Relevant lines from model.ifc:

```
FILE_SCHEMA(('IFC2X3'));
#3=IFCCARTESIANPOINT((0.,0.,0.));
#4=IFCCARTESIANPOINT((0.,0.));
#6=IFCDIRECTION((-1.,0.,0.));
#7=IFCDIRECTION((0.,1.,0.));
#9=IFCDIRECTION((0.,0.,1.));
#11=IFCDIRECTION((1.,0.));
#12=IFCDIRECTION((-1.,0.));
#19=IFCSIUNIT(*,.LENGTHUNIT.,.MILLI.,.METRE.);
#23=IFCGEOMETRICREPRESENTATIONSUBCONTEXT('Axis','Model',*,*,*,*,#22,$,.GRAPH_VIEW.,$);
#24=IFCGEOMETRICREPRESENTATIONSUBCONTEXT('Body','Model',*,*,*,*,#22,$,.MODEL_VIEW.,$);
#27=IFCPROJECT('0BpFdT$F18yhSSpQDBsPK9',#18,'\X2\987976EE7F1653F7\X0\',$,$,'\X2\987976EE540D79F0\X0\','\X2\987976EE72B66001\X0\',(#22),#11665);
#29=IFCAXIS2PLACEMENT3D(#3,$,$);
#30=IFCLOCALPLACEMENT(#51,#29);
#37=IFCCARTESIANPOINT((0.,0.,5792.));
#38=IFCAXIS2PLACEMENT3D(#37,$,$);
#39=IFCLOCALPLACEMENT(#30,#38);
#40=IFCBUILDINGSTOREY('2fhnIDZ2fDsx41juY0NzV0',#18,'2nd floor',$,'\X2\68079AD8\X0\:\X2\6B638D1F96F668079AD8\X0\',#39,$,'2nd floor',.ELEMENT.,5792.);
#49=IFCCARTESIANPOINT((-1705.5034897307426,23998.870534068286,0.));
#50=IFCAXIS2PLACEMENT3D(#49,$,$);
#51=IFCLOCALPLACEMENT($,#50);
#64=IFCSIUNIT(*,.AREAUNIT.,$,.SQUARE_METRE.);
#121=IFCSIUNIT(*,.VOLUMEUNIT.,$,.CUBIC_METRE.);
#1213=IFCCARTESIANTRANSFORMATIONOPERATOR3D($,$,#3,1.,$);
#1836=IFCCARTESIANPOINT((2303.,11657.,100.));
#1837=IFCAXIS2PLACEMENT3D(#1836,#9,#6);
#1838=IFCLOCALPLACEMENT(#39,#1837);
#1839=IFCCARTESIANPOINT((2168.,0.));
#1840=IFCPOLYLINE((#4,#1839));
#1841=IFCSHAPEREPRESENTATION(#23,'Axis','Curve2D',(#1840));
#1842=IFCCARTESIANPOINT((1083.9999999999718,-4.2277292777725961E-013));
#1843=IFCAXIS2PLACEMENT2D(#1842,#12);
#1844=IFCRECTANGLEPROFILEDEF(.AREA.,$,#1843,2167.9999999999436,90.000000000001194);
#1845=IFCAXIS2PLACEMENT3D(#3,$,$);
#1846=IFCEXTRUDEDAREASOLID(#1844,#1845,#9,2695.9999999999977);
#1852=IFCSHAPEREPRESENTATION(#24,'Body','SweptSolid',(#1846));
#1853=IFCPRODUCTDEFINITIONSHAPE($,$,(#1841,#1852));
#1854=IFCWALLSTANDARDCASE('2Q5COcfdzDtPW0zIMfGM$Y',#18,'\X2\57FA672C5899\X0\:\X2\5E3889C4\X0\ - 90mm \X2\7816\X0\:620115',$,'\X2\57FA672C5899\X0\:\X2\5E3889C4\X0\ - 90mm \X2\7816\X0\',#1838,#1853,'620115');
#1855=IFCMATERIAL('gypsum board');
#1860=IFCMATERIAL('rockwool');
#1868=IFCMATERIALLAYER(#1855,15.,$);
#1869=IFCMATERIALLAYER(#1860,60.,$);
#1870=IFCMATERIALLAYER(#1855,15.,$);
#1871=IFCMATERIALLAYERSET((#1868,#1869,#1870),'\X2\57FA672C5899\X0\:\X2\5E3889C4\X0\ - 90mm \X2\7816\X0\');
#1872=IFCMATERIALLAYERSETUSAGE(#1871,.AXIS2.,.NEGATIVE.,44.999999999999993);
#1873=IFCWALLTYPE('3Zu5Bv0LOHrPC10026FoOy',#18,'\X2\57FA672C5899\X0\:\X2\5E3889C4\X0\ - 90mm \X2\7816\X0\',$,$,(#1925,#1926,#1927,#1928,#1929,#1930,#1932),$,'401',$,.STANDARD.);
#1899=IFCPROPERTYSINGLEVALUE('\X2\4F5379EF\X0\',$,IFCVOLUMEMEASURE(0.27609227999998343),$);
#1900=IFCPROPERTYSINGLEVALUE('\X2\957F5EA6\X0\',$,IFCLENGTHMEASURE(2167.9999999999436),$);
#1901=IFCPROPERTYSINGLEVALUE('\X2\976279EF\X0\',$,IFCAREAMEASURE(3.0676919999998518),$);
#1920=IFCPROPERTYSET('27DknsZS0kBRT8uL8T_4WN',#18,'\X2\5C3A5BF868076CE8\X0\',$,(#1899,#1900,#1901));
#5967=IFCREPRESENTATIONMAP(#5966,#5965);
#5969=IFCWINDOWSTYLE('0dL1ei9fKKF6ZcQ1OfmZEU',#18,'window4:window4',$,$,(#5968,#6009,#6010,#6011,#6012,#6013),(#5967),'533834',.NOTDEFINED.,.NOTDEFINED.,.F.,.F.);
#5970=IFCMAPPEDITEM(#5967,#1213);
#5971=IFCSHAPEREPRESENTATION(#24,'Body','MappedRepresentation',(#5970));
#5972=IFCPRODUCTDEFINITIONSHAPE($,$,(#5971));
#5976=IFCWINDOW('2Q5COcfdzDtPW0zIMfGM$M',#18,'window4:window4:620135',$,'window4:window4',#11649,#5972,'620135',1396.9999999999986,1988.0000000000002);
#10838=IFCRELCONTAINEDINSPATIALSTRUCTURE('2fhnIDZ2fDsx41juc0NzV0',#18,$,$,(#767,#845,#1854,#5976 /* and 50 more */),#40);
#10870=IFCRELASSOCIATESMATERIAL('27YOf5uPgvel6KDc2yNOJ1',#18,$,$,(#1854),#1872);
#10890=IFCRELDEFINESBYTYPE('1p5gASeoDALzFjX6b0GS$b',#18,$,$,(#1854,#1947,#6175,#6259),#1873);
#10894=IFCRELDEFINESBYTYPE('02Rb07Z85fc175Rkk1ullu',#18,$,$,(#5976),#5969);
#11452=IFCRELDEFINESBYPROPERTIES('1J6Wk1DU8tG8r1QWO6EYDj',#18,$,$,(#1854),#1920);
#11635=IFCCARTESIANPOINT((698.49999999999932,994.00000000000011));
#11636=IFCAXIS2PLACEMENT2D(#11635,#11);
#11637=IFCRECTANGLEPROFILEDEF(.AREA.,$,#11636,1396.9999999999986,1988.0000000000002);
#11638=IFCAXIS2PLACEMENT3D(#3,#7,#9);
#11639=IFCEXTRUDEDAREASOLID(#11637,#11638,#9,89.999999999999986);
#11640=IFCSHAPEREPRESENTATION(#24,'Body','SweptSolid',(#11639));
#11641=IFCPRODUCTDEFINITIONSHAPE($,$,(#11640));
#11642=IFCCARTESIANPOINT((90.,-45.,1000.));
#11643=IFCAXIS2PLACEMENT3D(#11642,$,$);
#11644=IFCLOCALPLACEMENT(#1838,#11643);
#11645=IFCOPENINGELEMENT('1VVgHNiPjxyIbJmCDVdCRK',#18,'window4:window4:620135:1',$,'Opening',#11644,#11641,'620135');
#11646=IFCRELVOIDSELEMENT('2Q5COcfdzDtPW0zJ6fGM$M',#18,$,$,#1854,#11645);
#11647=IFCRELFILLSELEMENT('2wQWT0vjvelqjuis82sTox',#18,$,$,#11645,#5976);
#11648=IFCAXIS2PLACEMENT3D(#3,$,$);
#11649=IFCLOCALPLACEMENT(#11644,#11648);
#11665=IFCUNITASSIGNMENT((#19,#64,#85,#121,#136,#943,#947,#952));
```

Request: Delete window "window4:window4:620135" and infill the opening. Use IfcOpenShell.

```python
import ifcopenshell
import ifcopenshell.api.feature
import ifcopenshell.api.pset
import ifcopenshell.api.root
import ifcopenshell.geom
import ifcopenshell.util.element
import ifcopenshell.util.shape
import ifcopenshell.util.unit

model = ifcopenshell.open("model.ifc")
area_scale = ifcopenshell.util.unit.calculate_unit_scale(model, "AREAUNIT")
volume_scale = ifcopenshell.util.unit.calculate_unit_scale(model, "VOLUMEUNIT")
settings = ifcopenshell.geom.settings()


def volume(element):
    """Net volume in cubic metres, openings subtracted."""
    shape = ifcopenshell.geom.create_shape(settings, element)
    return ifcopenshell.util.shape.get_volume(shape.geometry)


window = model.by_guid("2Q5COcfdzDtPW0zIMfGM$M")
opening = window.FillsVoids[0].RelatingOpeningElement
wall = opening.VoidsElements[0].RelatingBuildingElement
before = volume(wall)

ifcopenshell.api.root.remove_product(model, product=window)
ifcopenshell.api.feature.remove_feature(model, feature=opening)

after = volume(wall)
thickness = 0.09  # wall thickness in metres

# Update the wall's stored quantities.
pset = model.by_id(ifcopenshell.util.element.get_pset(wall, "尺寸标注", should_inherit=False)["id"])
ifcopenshell.api.pset.edit_pset(model, pset=pset, properties={
    "体积": model.create_entity("IfcVolumeMeasure", after / volume_scale),
    "面积": model.create_entity("IfcAreaMeasure", after / thickness / area_scale),
})

print(f"wall volume {before:.3f} -> {after:.3f} m3")

model.write("model_edited.ifc")
```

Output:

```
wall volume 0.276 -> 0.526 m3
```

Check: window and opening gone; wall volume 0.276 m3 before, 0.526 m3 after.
